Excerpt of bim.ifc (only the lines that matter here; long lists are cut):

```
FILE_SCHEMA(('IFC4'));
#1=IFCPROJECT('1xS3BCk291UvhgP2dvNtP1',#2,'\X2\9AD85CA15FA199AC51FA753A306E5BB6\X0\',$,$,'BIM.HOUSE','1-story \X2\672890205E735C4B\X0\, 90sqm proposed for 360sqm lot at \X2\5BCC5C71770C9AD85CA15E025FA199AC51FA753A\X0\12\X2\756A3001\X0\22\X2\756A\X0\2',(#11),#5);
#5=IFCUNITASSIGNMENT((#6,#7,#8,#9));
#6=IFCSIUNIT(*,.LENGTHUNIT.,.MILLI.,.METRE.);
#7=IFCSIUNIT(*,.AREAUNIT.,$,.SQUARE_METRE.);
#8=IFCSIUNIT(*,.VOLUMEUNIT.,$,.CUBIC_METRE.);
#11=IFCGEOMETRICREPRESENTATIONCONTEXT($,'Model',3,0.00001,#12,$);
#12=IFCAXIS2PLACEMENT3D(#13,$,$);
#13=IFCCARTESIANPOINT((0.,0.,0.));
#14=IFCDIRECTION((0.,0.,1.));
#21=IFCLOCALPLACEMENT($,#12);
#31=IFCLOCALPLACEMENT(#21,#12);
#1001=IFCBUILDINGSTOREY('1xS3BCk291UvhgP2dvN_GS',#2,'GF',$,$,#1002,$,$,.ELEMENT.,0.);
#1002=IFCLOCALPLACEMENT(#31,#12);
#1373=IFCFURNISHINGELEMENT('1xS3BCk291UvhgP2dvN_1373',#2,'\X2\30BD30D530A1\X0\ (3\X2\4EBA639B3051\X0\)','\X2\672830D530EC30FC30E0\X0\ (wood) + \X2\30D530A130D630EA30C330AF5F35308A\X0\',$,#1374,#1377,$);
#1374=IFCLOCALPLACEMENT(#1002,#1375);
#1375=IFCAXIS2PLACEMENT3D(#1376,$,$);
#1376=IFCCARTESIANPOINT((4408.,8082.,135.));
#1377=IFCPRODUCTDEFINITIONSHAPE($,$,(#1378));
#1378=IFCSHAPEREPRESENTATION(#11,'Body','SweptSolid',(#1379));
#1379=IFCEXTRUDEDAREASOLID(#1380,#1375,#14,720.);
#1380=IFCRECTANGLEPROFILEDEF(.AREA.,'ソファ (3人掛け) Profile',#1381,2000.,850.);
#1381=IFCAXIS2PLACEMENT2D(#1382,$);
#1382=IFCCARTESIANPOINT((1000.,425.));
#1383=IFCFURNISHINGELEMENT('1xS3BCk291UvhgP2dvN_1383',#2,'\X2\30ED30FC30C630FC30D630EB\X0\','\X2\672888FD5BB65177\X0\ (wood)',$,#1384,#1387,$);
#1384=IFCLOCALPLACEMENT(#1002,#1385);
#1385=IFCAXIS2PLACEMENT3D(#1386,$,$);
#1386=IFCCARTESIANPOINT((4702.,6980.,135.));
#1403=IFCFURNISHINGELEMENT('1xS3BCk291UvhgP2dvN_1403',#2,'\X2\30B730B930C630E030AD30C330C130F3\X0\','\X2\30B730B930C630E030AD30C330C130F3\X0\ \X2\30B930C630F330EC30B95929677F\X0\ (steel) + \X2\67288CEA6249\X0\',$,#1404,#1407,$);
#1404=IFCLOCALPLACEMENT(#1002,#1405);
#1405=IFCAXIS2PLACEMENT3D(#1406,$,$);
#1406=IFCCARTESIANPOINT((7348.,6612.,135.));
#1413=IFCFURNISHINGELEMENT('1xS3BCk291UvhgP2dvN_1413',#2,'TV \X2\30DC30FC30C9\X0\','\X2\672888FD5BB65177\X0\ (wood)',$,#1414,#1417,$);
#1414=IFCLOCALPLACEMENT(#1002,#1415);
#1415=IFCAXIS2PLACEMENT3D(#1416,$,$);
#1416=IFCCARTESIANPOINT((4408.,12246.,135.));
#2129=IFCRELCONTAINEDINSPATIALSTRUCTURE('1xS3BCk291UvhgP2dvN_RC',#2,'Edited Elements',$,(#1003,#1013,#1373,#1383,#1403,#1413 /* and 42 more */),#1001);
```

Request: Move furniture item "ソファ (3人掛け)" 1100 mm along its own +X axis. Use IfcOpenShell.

```python
import ifcopenshell
import ifcopenshell.api.geometry
import ifcopenshell.util.placement
import ifcopenshell.util.unit

model = ifcopenshell.open("bim.ifc")
unit_scale = ifcopenshell.util.unit.calculate_unit_scale(model)

item = model.by_id(1373)
matrix = ifcopenshell.util.placement.get_local_placement(item.ObjectPlacement)
matrix[:3, 3] += matrix[:3, 0] * 1.1 / unit_scale
ifcopenshell.api.geometry.edit_object_placement(model, product=item, matrix=matrix, is_si=False)

print(ifcopenshell.util.placement.get_local_placement(item.ObjectPlacement).round(3) + 0.0)

model.write("bim_rev.ifc")
```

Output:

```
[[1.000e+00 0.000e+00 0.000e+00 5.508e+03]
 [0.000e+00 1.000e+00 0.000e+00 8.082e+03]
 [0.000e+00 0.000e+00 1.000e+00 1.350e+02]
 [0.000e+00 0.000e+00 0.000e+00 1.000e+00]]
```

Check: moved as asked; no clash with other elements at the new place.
